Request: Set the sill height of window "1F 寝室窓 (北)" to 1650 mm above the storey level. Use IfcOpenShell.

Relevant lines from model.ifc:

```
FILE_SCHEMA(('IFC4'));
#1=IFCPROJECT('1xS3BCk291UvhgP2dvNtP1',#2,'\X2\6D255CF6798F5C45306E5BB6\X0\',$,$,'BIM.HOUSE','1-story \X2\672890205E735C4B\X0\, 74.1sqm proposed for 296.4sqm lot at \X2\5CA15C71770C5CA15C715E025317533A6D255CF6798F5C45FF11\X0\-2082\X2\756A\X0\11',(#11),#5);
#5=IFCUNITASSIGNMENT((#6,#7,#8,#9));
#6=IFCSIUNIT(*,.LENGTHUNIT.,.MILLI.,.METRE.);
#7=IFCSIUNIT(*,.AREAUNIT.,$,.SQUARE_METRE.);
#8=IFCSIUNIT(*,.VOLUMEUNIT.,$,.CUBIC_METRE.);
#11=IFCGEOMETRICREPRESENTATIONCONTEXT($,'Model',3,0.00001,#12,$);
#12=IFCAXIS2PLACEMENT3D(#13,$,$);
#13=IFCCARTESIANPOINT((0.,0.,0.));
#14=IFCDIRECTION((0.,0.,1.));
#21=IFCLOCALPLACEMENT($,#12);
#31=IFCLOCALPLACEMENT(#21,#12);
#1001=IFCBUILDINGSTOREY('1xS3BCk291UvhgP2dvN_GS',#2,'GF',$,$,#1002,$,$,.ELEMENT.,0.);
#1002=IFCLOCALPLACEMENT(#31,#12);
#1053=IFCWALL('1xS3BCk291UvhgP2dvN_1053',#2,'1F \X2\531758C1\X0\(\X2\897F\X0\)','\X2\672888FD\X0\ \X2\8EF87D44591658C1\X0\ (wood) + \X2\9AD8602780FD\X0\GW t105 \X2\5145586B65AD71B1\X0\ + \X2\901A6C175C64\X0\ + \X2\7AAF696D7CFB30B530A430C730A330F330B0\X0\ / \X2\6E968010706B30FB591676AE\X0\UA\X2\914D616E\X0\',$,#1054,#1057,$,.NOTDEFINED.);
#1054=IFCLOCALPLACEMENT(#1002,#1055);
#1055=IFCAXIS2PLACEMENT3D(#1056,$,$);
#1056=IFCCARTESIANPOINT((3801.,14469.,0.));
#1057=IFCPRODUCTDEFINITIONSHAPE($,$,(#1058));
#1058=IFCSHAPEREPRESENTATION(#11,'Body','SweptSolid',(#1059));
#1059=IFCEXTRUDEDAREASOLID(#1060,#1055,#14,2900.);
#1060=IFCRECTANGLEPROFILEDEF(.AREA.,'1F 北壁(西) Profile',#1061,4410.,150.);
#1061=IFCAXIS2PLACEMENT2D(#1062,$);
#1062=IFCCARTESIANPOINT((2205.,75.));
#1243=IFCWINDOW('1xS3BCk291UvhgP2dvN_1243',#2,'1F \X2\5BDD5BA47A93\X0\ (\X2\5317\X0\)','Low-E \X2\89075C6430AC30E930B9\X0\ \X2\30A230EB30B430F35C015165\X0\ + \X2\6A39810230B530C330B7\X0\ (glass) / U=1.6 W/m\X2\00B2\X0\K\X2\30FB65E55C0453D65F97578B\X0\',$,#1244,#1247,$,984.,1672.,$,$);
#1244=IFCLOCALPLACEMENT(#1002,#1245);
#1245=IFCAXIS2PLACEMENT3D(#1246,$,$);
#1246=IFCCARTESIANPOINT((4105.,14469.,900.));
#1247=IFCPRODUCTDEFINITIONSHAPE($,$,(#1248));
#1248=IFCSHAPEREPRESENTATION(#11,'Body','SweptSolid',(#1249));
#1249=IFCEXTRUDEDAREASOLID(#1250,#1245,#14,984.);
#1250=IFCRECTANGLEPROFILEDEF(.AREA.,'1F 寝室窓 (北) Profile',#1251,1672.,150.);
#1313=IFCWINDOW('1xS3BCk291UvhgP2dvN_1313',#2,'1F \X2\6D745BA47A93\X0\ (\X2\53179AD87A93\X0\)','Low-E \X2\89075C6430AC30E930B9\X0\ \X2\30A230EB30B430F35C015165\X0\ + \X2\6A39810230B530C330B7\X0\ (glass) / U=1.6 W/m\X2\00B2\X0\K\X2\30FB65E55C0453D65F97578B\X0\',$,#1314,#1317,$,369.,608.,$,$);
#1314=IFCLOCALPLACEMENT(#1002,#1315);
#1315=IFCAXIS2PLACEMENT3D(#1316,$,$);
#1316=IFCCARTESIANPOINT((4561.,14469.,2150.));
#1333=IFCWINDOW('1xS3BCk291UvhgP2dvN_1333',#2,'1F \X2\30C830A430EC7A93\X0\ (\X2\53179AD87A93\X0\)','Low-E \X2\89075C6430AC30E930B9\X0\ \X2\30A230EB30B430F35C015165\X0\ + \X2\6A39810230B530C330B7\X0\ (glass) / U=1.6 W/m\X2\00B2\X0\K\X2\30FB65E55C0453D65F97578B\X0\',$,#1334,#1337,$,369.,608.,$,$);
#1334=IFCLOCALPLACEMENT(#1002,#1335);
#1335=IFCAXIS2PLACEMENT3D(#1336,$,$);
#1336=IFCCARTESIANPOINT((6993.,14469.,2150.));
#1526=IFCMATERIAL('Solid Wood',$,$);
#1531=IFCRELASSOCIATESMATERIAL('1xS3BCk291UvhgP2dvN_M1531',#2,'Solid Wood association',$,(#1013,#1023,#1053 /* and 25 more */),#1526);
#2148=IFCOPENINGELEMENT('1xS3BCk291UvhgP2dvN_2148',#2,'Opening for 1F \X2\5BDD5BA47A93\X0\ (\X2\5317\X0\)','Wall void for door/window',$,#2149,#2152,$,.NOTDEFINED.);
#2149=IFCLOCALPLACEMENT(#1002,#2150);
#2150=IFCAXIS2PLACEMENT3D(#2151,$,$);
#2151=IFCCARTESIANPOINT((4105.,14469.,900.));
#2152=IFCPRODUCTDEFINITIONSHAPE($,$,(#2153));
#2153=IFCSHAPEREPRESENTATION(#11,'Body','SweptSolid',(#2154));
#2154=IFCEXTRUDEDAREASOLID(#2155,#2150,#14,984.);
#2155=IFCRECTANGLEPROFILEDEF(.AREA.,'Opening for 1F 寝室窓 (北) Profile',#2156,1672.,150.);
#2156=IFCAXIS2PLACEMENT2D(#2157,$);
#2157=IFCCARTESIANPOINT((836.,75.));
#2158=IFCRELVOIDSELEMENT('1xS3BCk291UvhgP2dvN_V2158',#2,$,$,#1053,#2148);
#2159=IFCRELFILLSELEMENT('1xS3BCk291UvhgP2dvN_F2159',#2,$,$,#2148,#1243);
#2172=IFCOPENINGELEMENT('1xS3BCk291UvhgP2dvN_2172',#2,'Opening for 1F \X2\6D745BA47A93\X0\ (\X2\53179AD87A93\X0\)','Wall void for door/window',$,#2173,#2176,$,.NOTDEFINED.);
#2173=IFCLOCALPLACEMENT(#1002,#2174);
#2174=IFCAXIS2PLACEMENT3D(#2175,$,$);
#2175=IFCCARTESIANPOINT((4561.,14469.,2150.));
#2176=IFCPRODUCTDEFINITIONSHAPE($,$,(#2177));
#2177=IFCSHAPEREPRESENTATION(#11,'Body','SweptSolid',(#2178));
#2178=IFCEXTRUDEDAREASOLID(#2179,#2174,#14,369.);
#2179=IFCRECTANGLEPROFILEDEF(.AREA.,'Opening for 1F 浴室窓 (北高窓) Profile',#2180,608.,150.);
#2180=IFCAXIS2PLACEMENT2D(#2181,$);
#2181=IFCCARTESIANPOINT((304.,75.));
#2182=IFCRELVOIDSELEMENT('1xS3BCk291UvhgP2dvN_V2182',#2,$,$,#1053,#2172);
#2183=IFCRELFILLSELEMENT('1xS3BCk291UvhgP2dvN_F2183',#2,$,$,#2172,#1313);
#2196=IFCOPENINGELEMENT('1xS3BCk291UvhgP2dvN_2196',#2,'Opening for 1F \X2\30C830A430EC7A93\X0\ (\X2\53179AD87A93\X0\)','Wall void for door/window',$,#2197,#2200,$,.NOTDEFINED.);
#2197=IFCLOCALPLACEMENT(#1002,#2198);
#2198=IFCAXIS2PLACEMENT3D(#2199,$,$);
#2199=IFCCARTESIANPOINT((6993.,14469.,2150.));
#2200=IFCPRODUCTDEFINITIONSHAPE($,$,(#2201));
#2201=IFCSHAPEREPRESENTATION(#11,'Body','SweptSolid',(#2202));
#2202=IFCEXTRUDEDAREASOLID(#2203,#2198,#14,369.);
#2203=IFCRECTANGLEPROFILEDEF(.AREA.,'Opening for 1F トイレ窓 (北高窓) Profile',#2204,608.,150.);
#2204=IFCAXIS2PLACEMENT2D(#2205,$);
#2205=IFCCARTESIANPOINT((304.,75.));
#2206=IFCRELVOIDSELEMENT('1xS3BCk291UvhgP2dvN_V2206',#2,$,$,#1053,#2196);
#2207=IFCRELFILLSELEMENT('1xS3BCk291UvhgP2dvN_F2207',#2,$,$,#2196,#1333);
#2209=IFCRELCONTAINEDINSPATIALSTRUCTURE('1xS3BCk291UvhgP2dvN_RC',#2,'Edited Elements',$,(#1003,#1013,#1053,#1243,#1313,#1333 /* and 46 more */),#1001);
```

```python
import numpy as np
import ifcopenshell
import ifcopenshell.api.geometry
import ifcopenshell.geom
import ifcopenshell.util.element
import ifcopenshell.util.placement
import ifcopenshell.util.shape
import ifcopenshell.util.unit

model = ifcopenshell.open("model.ifc")
unit_scale = ifcopenshell.util.unit.calculate_unit_scale(model)

window = model.by_guid("1xS3BCk291UvhgP2dvN_1243")
opening = window.FillsVoids[0].RelatingOpeningElement
storey = ifcopenshell.util.element.get_container(window, ifc_class="IfcBuildingStorey")
level = ifcopenshell.util.placement.get_local_placement(storey.ObjectPlacement)[2, 3]

# The opening's origin need not be at the sill, so measure its lowest point.
shape = ifcopenshell.geom.create_shape(ifcopenshell.geom.settings(), opening)
bottom = ifcopenshell.util.shape.get_shape_bottom_elevation(shape, shape.geometry) / unit_scale
dz = level + 1.65 / unit_scale - bottom

shift = np.array([0.0, 0.0, dz])
# The window is not placed relative to its opening, so move both.
for product in (opening, window):
    matrix = ifcopenshell.util.placement.get_local_placement(product.ObjectPlacement)
    matrix[:3, 3] += shift
    ifcopenshell.api.geometry.edit_object_placement(model, product=product, matrix=matrix, is_si=False)

print(f"moved by {dz * unit_scale:+.3f} m")

model.write("model_updated.ifc")
```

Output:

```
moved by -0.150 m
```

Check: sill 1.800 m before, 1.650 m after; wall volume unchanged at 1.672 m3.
